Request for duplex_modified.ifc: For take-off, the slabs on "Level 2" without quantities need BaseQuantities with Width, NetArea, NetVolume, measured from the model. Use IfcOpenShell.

First a look at what the model holds.

```python
import ifcopenshell
import ifcopenshell.util.element
import ifcopenshell.util.unit

model = ifcopenshell.open("duplex_modified.ifc")
print(model.schema)
for unit_type in ("LENGTHUNIT", "AREAUNIT", "VOLUMEUNIT"):
    print(unit_type, ifcopenshell.util.unit.calculate_unit_scale(model, unit_type))
storey = next(s for s in model.by_type("IfcBuildingStorey") if s.Name == "Level 2")
slabs = [e for e in ifcopenshell.util.element.get_decomposition(storey) if e.is_a("IfcSlab")]
for e in sorted(slabs, key=lambda e: e.id()):
    print(e.id(), e.is_a(), e.Name, list(ifcopenshell.util.element.get_psets(e, qtos_only=True)), sep=" | ")
```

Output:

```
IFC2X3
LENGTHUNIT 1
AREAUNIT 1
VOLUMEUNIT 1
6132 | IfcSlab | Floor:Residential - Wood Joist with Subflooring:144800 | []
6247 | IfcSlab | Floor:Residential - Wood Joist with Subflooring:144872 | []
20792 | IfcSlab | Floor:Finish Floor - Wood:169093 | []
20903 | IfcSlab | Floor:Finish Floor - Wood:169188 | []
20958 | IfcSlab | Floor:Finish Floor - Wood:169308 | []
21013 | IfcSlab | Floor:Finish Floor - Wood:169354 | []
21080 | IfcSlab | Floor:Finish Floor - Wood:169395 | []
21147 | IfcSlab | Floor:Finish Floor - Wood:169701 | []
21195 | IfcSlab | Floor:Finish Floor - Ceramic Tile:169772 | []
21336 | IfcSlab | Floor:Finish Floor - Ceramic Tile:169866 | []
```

```python
import ifcopenshell
import ifcopenshell.api.pset
import ifcopenshell.geom
import ifcopenshell.util.element
import ifcopenshell.util.shape
import ifcopenshell.util.unit

model = ifcopenshell.open("duplex_modified.ifc")
unit_scale = ifcopenshell.util.unit.calculate_unit_scale(model)
area_scale = ifcopenshell.util.unit.calculate_unit_scale(model, "AREAUNIT")
volume_scale = ifcopenshell.util.unit.calculate_unit_scale(model, "VOLUMEUNIT")
settings = ifcopenshell.geom.settings()

storey = next(s for s in model.by_type("IfcBuildingStorey") if s.Name == "Level 2")
slabs = [e for e in ifcopenshell.util.element.get_decomposition(storey) if e.is_a("IfcSlab")]

for e in sorted(slabs, key=lambda e: e.id()):
    if ifcopenshell.util.element.get_psets(e, qtos_only=True, should_inherit=False):
        continue
    # Geometry comes back in metres, in the element's own axes.
    shape = ifcopenshell.geom.create_shape(settings, e)
    values = {
        "Width": ifcopenshell.util.shape.get_z(shape.geometry) / unit_scale,
        "NetArea": ifcopenshell.util.shape.get_footprint_area(shape.geometry) / area_scale,
        "NetVolume": ifcopenshell.util.shape.get_volume(shape.geometry) / volume_scale,
    }
    qto = ifcopenshell.api.pset.add_qto(model, product=e, name="BaseQuantities")
    ifcopenshell.api.pset.edit_qto(model, qto=qto, properties=values)
    print(e.id(), {k: round(v, 3) for k, v in values.items()})

model.write("duplex_modified-out.ifc")
```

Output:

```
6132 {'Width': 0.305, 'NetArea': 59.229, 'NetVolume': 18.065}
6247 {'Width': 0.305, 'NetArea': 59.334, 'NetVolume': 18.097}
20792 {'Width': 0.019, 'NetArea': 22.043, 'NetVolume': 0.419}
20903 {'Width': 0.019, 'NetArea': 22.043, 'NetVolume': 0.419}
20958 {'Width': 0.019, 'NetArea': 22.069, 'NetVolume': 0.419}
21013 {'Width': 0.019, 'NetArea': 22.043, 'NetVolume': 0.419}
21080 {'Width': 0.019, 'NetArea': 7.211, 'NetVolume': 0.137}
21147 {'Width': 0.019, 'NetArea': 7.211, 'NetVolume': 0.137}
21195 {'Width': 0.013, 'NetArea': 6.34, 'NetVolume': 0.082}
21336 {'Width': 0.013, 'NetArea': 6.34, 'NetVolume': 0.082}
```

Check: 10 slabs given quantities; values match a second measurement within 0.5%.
